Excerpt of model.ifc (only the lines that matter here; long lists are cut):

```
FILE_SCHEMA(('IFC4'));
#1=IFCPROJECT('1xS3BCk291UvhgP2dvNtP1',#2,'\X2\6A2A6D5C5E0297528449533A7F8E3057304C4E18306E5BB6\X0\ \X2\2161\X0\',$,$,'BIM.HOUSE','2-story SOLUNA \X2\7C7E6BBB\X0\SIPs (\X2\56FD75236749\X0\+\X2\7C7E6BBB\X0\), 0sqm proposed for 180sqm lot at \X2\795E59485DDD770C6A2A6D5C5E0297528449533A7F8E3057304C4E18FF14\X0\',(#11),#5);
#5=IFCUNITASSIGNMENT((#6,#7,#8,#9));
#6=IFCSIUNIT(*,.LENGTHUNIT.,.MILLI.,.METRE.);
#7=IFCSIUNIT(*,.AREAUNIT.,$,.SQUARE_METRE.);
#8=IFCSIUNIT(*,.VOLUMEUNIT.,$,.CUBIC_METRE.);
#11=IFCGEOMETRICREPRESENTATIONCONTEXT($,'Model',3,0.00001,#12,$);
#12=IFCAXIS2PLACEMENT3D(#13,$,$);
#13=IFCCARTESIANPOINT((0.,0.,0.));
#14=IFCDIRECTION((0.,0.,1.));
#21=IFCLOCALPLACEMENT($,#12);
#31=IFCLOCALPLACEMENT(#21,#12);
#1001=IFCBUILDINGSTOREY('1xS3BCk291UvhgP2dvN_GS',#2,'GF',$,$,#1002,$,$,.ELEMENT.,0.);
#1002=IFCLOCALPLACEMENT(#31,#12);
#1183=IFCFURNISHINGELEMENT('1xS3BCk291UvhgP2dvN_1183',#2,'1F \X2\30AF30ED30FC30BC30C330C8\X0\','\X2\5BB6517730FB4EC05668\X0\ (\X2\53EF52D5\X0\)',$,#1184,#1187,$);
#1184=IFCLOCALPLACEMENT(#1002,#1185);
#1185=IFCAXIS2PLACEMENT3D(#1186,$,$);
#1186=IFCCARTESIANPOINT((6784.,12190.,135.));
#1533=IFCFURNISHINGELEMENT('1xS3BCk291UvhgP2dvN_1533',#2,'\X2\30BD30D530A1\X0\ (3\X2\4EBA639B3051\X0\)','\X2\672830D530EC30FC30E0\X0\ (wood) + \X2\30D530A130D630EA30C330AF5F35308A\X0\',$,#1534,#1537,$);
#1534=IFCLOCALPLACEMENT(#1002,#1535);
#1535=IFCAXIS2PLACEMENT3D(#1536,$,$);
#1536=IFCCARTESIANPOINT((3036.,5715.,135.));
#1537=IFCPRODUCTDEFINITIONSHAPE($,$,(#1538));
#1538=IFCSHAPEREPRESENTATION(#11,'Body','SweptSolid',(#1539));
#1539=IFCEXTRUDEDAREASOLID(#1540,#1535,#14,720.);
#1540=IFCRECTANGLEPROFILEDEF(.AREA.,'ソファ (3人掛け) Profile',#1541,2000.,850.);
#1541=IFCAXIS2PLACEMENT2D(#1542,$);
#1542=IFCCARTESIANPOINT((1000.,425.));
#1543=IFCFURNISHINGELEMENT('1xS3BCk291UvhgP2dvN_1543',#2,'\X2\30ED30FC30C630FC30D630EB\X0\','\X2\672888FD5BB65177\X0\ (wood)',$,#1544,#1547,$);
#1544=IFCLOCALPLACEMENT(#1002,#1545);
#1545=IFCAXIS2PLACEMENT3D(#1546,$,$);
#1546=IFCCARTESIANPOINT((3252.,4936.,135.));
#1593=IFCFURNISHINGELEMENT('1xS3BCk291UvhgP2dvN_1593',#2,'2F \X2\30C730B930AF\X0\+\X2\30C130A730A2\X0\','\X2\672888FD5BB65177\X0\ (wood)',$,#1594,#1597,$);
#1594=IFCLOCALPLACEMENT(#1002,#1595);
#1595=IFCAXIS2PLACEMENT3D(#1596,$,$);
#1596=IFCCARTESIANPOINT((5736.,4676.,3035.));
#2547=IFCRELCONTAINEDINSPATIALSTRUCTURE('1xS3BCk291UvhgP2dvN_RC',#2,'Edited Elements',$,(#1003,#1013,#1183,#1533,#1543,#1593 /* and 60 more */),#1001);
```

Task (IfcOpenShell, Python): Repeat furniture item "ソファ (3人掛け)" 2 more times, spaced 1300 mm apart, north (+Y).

```python
import numpy as np
import ifcopenshell
import ifcopenshell.api.geometry
import ifcopenshell.api.root
import ifcopenshell.util.element
import ifcopenshell.util.placement
import ifcopenshell.util.unit

model = ifcopenshell.open("model.ifc")
unit_scale = ifcopenshell.util.unit.calculate_unit_scale(model)


def reuse_history(source, copy):
    """copy_class also copies each property set's owner history, people and application; keep the originals."""
    for rel in copy.IsDefinedBy:
        if rel.is_a("IfcRelDefinesByProperties") and (history := rel.RelatingPropertyDefinition.OwnerHistory):
            rel.RelatingPropertyDefinition.OwnerHistory = source.OwnerHistory
            ifcopenshell.util.element.remove_deep2(model, history)


source = model.by_guid("1xS3BCk291UvhgP2dvN_1533")
base = ifcopenshell.util.placement.get_local_placement(source.ObjectPlacement)
step = np.array([0.0, 1.0, 0.0]) * 1.3 / unit_scale

for i in range(1, 3):
    copy = ifcopenshell.api.root.copy_class(model, product=source)
    copy.Representation = ifcopenshell.util.element.copy_deep(
        model, source.Representation, exclude=["IfcGeometricRepresentationContext", "IfcRepresentationMap"]
    )
    reuse_history(source, copy)
    matrix = base.copy()
    matrix[:3, 3] += i * step
    print("added at", matrix[:3, 3].round(3) + 0.0)
    ifcopenshell.api.geometry.edit_object_placement(model, product=copy, matrix=matrix, is_si=False)

model.write("model_v2.ifc")
```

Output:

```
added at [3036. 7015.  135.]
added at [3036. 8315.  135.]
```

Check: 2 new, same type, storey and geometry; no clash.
